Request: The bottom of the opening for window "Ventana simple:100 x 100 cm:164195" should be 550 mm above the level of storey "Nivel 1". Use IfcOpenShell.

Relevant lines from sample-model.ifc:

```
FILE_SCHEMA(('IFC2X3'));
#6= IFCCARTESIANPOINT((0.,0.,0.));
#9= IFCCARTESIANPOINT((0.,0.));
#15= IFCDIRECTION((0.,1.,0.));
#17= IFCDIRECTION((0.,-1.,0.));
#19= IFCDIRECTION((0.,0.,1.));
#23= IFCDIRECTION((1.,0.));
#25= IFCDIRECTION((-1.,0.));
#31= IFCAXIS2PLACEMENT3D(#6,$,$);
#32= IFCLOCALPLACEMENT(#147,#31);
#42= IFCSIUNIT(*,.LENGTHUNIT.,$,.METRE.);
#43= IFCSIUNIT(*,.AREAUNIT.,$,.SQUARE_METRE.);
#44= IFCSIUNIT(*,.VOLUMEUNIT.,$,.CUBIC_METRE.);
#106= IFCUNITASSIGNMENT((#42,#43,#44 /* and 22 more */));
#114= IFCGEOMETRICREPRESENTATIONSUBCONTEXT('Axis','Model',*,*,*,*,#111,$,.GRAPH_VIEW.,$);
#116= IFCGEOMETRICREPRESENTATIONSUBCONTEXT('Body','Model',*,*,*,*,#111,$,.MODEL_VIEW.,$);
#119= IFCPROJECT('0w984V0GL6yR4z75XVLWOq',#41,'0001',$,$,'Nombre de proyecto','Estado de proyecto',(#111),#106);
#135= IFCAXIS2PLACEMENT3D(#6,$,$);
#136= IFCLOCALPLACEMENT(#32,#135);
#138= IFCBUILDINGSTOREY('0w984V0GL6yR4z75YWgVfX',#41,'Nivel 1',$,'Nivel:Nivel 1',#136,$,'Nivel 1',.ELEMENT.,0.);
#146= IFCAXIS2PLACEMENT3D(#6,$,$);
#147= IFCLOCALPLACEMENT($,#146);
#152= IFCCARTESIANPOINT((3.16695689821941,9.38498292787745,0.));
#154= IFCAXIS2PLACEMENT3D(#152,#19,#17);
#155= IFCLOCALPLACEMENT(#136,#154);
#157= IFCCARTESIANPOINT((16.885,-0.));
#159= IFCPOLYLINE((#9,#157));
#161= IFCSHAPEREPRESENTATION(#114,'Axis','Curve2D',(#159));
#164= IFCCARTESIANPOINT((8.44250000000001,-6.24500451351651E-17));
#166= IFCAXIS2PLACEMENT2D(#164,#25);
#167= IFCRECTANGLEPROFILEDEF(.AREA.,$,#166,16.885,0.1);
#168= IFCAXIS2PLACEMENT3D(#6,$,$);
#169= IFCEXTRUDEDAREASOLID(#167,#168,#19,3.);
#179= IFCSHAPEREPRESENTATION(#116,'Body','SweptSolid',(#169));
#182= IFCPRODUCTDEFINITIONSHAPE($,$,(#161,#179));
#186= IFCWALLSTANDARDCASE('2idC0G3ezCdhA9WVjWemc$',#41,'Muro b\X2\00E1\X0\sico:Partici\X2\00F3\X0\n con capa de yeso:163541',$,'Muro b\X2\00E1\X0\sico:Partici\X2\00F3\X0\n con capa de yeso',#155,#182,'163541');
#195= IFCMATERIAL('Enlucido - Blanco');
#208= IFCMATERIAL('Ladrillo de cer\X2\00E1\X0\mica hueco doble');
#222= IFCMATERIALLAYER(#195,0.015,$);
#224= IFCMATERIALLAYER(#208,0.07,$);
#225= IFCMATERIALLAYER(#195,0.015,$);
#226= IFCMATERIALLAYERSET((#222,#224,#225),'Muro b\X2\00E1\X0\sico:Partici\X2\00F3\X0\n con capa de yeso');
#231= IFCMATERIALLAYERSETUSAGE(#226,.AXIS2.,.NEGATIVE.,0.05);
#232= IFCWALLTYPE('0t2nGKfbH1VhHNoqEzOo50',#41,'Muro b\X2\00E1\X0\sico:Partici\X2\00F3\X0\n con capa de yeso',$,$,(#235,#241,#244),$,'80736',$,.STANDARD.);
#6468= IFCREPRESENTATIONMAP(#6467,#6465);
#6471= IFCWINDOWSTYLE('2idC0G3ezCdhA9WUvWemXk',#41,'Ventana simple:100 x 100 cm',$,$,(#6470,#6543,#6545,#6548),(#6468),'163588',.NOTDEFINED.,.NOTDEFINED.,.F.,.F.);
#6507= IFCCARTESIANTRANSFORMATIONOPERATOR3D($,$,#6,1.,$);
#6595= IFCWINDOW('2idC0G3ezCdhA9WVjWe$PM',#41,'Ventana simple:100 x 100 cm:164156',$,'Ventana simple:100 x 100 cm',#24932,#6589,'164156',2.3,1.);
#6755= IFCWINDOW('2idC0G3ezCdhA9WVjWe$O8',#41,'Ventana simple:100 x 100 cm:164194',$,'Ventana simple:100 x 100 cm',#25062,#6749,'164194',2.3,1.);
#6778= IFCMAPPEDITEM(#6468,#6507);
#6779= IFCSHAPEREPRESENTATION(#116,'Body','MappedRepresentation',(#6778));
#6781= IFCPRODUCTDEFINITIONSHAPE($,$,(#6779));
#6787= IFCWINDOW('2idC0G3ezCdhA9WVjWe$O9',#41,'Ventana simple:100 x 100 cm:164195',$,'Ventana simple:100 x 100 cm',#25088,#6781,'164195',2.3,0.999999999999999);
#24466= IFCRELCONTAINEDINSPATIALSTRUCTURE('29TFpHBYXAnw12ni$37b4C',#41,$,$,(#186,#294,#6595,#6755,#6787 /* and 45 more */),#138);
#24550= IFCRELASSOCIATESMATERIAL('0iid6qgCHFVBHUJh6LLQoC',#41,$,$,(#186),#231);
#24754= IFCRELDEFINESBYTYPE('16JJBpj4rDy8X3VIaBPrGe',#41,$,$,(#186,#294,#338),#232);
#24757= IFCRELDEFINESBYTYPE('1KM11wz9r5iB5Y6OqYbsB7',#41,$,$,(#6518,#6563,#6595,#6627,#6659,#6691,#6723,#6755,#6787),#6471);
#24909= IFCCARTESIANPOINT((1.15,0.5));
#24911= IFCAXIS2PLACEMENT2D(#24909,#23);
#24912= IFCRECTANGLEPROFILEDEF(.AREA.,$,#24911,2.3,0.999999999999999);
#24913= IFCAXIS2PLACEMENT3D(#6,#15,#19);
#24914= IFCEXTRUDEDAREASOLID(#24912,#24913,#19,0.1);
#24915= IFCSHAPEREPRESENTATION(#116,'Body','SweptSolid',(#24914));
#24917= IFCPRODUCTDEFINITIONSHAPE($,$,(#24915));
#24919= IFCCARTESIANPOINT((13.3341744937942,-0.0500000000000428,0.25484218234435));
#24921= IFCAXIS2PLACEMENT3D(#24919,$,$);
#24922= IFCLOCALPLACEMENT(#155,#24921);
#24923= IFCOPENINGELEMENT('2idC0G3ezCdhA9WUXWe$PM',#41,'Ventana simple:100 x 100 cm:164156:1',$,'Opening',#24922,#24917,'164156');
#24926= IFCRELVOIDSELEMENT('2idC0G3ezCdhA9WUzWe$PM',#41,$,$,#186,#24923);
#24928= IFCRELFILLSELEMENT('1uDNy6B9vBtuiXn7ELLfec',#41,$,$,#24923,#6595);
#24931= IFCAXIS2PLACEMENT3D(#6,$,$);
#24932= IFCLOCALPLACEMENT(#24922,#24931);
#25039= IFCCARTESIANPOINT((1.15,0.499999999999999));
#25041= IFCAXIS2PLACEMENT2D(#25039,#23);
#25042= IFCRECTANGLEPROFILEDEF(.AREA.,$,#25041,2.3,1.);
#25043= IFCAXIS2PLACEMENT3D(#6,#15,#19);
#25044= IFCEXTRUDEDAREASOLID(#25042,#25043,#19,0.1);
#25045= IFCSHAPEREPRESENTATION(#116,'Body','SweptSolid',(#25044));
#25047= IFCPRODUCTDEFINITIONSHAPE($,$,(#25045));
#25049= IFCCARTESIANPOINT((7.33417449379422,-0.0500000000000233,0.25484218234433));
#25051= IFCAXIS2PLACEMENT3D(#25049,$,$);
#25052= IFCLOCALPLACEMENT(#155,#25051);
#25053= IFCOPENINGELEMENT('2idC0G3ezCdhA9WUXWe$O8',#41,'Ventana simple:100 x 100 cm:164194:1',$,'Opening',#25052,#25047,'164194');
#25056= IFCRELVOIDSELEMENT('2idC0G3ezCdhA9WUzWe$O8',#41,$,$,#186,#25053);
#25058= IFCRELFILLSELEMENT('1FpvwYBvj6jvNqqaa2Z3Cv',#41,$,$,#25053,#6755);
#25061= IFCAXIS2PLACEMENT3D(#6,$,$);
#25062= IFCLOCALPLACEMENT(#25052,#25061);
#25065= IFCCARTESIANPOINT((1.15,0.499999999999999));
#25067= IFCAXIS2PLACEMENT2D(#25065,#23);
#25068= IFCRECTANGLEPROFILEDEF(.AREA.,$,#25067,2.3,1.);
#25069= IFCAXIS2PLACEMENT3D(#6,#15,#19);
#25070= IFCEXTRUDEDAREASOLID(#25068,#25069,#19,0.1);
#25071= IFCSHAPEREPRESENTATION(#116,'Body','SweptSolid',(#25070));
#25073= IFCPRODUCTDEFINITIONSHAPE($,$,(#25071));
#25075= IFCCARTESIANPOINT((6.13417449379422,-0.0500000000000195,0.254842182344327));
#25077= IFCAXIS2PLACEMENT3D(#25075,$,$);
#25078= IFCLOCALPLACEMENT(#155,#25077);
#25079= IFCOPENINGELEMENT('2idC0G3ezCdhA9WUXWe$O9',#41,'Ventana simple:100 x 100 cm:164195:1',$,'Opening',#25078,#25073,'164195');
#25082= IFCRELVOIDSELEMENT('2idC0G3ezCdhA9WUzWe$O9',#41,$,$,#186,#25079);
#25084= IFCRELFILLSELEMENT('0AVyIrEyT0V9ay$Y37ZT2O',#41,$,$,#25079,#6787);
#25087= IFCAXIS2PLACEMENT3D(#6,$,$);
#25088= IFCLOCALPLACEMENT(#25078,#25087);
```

```python
import numpy as np
import ifcopenshell
import ifcopenshell.api.geometry
import ifcopenshell.geom
import ifcopenshell.util.element
import ifcopenshell.util.placement
import ifcopenshell.util.shape
import ifcopenshell.util.unit

model = ifcopenshell.open("sample-model.ifc")
unit_scale = ifcopenshell.util.unit.calculate_unit_scale(model)

window = model.by_guid("2idC0G3ezCdhA9WVjWe$O9")
opening = window.FillsVoids[0].RelatingOpeningElement
storey = ifcopenshell.util.element.get_container(window, ifc_class="IfcBuildingStorey")
level = ifcopenshell.util.placement.get_local_placement(storey.ObjectPlacement)[2, 3]

# The opening's origin need not be at the sill, so measure its lowest point.
shape = ifcopenshell.geom.create_shape(ifcopenshell.geom.settings(), opening)
bottom = ifcopenshell.util.shape.get_shape_bottom_elevation(shape, shape.geometry) / unit_scale
dz = level + 0.55 - bottom

shift = np.array([0.0, 0.0, dz])
# The window is placed relative to its opening, so it follows when the opening moves.
matrix = ifcopenshell.util.placement.get_local_placement(opening.ObjectPlacement)
matrix[:3, 3] += shift
ifcopenshell.api.geometry.edit_object_placement(
    model, product=opening, matrix=matrix, is_si=False, should_transform_children=True
)

print(f"moved by {dz * unit_scale:+.3f} m")

model.write("sample-model_updated.ifc")
```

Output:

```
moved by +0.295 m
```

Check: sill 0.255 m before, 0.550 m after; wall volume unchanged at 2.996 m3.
